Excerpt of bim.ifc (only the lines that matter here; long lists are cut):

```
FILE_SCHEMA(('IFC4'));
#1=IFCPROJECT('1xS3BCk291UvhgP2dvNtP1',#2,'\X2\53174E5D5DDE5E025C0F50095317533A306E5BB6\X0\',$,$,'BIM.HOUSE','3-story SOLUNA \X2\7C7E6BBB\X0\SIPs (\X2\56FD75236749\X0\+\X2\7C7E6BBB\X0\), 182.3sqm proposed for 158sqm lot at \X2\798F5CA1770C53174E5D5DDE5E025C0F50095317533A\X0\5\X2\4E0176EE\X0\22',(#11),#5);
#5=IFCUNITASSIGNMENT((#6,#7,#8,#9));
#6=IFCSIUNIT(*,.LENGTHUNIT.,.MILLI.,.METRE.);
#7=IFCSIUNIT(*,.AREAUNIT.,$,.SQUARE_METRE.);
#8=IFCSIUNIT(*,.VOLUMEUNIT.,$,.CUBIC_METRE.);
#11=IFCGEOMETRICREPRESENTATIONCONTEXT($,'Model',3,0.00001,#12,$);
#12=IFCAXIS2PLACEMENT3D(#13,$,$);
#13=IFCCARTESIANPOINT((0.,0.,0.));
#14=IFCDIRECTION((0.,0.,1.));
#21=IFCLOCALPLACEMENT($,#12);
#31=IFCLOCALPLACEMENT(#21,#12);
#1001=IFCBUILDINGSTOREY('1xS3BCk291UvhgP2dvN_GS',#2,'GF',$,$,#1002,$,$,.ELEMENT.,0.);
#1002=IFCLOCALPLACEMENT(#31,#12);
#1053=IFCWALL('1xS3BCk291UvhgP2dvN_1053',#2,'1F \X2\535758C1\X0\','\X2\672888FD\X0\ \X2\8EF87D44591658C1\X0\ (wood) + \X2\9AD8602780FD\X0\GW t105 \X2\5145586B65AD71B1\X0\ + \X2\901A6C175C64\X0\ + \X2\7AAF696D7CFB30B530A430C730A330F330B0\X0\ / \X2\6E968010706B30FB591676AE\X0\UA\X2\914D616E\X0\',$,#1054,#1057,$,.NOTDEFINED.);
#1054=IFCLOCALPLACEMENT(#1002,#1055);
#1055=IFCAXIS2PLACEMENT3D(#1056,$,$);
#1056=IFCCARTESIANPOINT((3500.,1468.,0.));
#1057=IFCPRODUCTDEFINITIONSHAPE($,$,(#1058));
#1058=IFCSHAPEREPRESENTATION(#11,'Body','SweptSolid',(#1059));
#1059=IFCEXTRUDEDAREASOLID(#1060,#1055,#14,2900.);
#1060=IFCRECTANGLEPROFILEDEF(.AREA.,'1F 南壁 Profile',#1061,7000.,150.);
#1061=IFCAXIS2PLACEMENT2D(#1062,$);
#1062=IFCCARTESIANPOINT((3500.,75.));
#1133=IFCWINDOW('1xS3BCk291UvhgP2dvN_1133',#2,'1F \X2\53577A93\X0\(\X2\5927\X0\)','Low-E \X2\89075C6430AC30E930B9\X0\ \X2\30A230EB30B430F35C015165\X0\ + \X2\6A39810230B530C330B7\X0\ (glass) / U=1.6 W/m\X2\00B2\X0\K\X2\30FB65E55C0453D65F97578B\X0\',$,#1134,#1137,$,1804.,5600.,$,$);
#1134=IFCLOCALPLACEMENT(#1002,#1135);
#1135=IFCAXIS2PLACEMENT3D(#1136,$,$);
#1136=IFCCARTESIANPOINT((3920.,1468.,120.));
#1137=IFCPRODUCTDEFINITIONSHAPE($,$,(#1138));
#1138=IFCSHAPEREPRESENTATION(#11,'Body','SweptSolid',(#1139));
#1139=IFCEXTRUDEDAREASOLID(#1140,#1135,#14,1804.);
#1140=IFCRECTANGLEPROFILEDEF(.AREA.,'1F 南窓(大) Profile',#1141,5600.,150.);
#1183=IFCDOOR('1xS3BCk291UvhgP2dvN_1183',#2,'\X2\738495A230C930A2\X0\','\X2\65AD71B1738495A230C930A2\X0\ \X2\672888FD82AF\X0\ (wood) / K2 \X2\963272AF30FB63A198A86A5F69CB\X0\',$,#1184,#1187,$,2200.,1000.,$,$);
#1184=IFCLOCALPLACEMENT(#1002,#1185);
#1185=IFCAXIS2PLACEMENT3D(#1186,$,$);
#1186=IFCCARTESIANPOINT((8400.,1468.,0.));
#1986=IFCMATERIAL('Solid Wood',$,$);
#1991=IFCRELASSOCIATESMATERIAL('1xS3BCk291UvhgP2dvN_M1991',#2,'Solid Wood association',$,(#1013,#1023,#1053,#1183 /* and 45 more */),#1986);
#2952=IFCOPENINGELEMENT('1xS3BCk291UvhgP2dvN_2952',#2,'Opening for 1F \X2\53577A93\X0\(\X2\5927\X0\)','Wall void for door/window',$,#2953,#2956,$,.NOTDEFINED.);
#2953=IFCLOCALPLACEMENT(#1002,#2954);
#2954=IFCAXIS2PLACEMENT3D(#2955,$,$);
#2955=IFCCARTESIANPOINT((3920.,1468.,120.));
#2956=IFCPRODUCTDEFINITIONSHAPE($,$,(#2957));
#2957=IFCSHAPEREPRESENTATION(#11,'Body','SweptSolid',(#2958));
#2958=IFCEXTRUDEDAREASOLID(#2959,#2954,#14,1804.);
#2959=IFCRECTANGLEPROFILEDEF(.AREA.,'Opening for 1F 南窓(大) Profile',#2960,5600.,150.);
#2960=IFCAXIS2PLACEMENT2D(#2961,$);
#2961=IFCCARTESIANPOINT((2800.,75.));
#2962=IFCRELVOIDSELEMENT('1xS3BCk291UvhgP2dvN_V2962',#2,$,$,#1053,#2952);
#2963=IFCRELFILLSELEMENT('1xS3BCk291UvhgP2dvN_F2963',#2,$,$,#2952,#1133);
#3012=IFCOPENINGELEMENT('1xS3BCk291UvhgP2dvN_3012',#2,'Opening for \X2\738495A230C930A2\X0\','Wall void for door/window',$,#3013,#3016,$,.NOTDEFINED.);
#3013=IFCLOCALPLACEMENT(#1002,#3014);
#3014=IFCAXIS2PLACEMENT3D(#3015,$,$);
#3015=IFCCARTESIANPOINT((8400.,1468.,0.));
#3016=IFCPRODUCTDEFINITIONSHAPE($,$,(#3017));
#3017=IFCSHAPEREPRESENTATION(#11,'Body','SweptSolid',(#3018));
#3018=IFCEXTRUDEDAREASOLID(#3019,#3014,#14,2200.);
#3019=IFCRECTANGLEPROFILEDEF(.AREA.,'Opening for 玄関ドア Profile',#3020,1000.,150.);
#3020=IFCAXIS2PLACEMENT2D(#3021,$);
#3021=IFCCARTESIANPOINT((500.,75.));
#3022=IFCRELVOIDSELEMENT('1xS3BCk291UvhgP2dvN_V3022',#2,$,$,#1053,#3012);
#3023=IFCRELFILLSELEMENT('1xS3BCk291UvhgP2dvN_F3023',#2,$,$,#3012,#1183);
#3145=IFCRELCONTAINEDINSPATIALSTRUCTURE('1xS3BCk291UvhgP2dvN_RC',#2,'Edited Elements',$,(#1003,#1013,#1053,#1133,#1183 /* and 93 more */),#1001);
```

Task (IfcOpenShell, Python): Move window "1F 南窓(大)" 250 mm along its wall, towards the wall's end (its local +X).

```python
import ifcopenshell
import ifcopenshell.api.geometry
import ifcopenshell.util.placement

model = ifcopenshell.open("bim.ifc")

window = model.by_guid("1xS3BCk291UvhgP2dvN_1133")
opening = window.FillsVoids[0].RelatingOpeningElement
wall = opening.VoidsElements[0].RelatingBuildingElement

wall_matrix = ifcopenshell.util.placement.get_local_placement(wall.ObjectPlacement)
shift = wall_matrix[:3, 0] * 250.0
before = ifcopenshell.util.placement.get_local_placement(window.ObjectPlacement)[:3, 3].copy()

# The window is not placed relative to its opening, so move both.
for product in (opening, window):
    matrix = ifcopenshell.util.placement.get_local_placement(product.ObjectPlacement)
    matrix[:3, 3] += shift
    ifcopenshell.api.geometry.edit_object_placement(model, product=product, matrix=matrix, is_si=False)

after = ifcopenshell.util.placement.get_local_placement(window.ObjectPlacement)[:3, 3]
print("window moved by", (after - before).round(3) + 0.0)

model.write("bim_rev.ifc")
```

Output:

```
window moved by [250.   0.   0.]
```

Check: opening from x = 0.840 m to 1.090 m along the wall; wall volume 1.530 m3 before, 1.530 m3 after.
